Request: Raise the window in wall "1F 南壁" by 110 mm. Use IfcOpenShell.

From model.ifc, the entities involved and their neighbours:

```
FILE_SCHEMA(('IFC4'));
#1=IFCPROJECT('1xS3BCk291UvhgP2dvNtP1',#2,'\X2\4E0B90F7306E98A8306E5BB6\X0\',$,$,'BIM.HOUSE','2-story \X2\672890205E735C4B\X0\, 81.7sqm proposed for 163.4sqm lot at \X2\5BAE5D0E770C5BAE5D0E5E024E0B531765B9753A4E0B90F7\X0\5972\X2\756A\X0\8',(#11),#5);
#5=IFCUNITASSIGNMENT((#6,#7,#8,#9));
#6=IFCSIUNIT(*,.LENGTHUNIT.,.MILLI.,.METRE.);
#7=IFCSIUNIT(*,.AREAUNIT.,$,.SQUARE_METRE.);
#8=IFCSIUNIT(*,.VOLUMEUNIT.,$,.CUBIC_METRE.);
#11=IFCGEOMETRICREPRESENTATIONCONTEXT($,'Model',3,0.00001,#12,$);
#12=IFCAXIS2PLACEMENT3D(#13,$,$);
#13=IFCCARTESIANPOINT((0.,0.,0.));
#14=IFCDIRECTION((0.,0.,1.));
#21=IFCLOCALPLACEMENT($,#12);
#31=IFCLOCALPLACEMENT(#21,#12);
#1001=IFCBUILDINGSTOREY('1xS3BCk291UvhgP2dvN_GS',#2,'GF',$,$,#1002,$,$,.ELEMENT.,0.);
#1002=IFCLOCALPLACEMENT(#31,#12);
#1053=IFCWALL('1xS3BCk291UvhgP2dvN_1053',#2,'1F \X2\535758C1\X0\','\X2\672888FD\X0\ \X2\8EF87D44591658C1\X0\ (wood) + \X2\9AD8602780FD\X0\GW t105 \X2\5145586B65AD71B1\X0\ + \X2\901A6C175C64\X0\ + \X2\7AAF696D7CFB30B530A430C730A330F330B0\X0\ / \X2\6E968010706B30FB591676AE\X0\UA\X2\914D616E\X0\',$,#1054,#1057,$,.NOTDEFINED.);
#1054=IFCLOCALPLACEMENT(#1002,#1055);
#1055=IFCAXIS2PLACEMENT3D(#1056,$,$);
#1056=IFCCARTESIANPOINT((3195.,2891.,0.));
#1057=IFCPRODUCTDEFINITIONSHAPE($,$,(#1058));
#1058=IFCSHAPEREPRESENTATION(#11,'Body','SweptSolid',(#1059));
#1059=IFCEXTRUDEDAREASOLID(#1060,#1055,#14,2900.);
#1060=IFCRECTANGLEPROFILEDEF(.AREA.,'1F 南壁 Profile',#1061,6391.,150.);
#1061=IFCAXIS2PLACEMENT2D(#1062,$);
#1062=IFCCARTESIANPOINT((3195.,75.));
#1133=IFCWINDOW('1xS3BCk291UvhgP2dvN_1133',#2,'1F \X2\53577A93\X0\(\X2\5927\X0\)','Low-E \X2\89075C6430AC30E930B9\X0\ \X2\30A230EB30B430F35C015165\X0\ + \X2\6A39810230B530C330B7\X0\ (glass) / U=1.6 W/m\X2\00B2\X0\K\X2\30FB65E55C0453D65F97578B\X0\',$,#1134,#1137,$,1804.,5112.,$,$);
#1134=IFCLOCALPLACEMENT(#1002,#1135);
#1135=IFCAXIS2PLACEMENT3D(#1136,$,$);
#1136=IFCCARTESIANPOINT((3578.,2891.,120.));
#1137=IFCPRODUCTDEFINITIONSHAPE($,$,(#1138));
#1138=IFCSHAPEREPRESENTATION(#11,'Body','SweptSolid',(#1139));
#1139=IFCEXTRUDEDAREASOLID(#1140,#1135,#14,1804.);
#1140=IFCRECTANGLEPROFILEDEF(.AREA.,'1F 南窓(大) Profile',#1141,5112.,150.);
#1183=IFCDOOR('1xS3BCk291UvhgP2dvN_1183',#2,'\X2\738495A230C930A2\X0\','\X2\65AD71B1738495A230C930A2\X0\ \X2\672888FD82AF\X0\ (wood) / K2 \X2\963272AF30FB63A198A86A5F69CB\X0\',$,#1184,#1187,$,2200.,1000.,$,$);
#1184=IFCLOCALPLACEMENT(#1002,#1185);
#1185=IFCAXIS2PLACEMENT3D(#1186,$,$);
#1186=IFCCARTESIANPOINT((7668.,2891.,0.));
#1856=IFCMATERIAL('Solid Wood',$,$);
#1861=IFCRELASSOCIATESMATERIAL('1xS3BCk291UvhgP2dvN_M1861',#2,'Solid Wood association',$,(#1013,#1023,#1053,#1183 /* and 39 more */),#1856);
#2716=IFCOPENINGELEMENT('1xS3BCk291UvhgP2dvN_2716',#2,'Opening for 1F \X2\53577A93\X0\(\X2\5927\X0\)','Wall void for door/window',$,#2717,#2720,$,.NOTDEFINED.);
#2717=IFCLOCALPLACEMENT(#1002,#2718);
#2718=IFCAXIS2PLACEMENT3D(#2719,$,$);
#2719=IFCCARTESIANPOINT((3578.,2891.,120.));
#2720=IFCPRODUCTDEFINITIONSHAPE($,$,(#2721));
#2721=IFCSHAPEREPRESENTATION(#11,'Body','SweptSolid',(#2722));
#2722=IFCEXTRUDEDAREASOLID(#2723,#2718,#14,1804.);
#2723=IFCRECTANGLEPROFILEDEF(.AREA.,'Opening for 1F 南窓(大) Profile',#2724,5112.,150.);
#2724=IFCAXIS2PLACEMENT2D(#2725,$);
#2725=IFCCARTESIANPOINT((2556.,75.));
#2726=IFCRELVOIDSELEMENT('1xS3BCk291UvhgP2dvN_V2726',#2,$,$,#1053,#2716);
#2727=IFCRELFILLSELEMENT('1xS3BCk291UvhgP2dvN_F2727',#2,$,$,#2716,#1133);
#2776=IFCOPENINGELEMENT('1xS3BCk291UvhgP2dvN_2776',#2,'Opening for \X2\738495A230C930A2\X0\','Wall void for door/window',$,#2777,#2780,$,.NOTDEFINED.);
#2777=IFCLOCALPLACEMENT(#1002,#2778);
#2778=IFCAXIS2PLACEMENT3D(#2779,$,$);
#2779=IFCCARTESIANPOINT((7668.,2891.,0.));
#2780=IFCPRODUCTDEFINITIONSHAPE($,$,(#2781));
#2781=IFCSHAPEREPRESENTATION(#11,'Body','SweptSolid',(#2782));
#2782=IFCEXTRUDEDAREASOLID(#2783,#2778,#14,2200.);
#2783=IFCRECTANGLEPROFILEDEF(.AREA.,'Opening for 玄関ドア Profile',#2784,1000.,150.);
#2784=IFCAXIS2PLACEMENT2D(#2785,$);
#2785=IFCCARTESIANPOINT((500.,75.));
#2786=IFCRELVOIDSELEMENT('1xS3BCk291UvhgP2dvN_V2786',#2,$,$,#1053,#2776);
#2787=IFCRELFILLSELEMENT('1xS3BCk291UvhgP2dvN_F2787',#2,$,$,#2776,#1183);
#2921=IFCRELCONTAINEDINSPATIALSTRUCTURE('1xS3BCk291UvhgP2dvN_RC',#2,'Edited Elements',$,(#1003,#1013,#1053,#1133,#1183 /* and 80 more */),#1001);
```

```python
import numpy as np
import ifcopenshell
import ifcopenshell.api.geometry
import ifcopenshell.util.placement
import ifcopenshell.util.unit

model = ifcopenshell.open("model.ifc")
unit_scale = ifcopenshell.util.unit.calculate_unit_scale(model)

window = model.by_id(1133)
opening = window.FillsVoids[0].RelatingOpeningElement
dz = 0.11 / unit_scale

shift = np.array([0.0, 0.0, dz])
# The window is not placed relative to its opening, so move both.
for product in (opening, window):
    matrix = ifcopenshell.util.placement.get_local_placement(product.ObjectPlacement)
    matrix[:3, 3] += shift
    ifcopenshell.api.geometry.edit_object_placement(model, product=product, matrix=matrix, is_si=False)

print(f"moved by {dz * unit_scale:+.3f} m")

model.write("model_edited.ifc")
```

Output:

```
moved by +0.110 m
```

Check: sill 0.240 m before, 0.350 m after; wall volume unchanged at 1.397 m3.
